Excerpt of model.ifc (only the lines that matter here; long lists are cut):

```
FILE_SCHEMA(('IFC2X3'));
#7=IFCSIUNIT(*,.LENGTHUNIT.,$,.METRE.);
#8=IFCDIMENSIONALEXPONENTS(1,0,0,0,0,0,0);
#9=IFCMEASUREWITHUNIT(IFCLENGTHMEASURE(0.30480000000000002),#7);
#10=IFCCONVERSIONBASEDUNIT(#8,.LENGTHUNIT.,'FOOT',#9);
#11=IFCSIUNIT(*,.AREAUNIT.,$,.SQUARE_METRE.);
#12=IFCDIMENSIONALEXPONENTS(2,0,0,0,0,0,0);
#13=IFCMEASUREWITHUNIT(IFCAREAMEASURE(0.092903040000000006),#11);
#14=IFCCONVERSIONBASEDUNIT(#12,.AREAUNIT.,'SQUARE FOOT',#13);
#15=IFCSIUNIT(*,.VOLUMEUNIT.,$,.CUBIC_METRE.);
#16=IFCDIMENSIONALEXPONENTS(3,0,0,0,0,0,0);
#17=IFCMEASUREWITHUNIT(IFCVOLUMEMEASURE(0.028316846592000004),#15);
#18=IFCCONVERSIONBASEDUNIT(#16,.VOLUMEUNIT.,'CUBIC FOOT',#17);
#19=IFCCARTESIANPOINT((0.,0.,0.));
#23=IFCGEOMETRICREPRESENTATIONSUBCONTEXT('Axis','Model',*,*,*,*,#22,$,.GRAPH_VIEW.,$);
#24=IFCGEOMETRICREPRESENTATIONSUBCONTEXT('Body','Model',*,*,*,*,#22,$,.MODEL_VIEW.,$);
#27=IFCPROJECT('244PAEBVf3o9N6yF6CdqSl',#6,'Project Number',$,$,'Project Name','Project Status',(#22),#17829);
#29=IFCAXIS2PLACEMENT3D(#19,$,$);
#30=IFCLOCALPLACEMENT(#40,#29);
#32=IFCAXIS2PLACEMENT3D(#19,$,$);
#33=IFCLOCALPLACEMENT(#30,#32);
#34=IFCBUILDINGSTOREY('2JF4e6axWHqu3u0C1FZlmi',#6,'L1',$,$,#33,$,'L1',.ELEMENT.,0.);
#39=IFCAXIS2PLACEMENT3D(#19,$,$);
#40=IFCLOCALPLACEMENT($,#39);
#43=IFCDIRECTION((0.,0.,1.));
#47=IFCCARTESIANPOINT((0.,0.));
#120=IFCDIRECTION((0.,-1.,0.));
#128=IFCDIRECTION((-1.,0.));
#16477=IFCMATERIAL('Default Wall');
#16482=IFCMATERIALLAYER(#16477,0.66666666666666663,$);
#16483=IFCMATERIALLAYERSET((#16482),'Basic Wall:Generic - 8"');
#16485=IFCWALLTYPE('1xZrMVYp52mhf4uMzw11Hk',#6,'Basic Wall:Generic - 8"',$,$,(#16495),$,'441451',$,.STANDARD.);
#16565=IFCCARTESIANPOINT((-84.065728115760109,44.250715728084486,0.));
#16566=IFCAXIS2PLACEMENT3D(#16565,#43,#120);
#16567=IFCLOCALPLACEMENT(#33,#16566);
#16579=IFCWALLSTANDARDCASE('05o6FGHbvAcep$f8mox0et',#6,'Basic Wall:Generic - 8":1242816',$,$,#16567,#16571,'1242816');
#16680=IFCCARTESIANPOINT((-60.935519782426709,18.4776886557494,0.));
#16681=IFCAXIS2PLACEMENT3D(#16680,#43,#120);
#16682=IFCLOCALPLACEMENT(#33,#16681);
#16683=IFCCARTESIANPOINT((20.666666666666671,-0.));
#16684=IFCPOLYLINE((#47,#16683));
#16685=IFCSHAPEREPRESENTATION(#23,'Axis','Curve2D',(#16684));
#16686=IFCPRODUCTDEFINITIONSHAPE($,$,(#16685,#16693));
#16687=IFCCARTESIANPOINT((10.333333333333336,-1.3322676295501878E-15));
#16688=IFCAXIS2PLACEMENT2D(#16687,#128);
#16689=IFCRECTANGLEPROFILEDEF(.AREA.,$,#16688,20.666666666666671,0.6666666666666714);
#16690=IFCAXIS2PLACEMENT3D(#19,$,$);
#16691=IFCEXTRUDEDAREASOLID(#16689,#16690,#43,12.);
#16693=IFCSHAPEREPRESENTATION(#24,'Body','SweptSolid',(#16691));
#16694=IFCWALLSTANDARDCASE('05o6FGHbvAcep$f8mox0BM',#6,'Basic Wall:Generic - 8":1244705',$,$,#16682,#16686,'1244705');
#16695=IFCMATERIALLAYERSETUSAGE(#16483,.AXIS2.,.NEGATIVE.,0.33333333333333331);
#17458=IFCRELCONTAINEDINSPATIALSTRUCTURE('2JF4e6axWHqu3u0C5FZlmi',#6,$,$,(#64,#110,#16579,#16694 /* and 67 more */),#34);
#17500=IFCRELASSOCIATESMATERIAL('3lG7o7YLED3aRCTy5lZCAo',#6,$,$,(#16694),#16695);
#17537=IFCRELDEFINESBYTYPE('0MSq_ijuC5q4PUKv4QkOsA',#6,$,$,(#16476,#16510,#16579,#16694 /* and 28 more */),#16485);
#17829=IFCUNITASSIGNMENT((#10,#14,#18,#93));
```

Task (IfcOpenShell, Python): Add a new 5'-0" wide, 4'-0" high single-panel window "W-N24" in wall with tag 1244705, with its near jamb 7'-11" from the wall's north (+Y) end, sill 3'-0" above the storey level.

```python
import numpy as np
import ifcopenshell
import ifcopenshell.api.feature
import ifcopenshell.api.geometry
import ifcopenshell.api.root
import ifcopenshell.api.spatial
import ifcopenshell.api.type
import ifcopenshell.geom
import ifcopenshell.util.element
import ifcopenshell.util.placement
import ifcopenshell.util.representation
import ifcopenshell.util.shape
import ifcopenshell.util.unit

model = ifcopenshell.open("model.ifc")
unit_scale = ifcopenshell.util.unit.calculate_unit_scale(model)
settings = ifcopenshell.geom.settings()


def volume(element):
    """Net volume in cubic metres, openings subtracted."""
    shape = ifcopenshell.geom.create_shape(settings, element)
    return ifcopenshell.util.shape.get_volume(shape.geometry)


wall = model.by_guid("05o6FGHbvAcep$f8mox0BM")
storey = ifcopenshell.util.element.get_container(wall, ifc_class="IfcBuildingStorey")
context = ifcopenshell.util.representation.get_context(model, "Model", "Body", "MODEL_VIEW")
before = volume(wall)

width, height, from_end, sill = 1.524, 1.2192, 2.413, 0.9144  # metres

# The wall runs along its own X axis, and the end named is its -X end.
wall_shape = ifcopenshell.geom.create_shape(settings, wall)
x, y, z = ifcopenshell.util.shape.get_vertices(wall_shape.geometry).T
start = x.min() + from_end
face, thickness = float(y.min()), float(y.max() - y.min())
wall_matrix = ifcopenshell.util.placement.get_local_placement(wall.ObjectPlacement)
level = ifcopenshell.util.placement.get_local_placement(storey.ObjectPlacement)[2, 3]


def in_wall(x, y):
    """Placement at x, y metres in the wall's axes, at sill height."""
    matrix = wall_matrix.copy()
    matrix[:, 3] = wall_matrix @ np.array([x / unit_scale, y / unit_scale, 0.0, 1.0])
    matrix[2, 3] = level + sill / unit_scale
    return matrix


# Opening: a box that overshoots both wall faces by 50 mm.
opening = ifcopenshell.api.root.create_entity(model, ifc_class="IfcOpeningElement")
box = ifcopenshell.api.geometry.add_wall_representation(
    model, context=context, length=width, height=height, thickness=thickness + 0.1
)
ifcopenshell.api.geometry.assign_representation(model, product=opening, representation=box)
ifcopenshell.api.geometry.edit_object_placement(model, product=opening, matrix=in_wall(start, face - 0.05), is_si=False)
ifcopenshell.api.feature.add_feature(model, feature=opening, element=wall)

window = ifcopenshell.api.root.create_entity(model, ifc_class="IfcWindow", name="W-N24")
window.OverallWidth, window.OverallHeight = width / unit_scale, height / unit_scale
body = ifcopenshell.api.geometry.add_window_representation(
    model,
    context=context,
    overall_width=window.OverallWidth,
    overall_height=window.OverallHeight,
    partition_type="SINGLE_PANEL",
)
ifcopenshell.api.geometry.assign_representation(model, product=window, representation=body)
ifcopenshell.api.spatial.assign_container(model, products=[window], relating_structure=storey)
fills = ifcopenshell.api.feature.add_filling(model, opening=opening, element=window)
fills.OwnerHistory = window.OwnerHistory  # required in IFC2X3

# IFC2X3 keeps the operation on the window style.
style = ifcopenshell.api.root.create_entity(model, ifc_class="IfcWindowStyle", name="W-N24")
style.OperationType, style.ConstructionType = "SINGLE_PANEL", "NOTDEFINED"
style.ParameterTakesPrecedence = style.Sizeable = False
ifcopenshell.api.type.assign_type(model, related_objects=[window], relating_type=style)

# Centre the window in the wall's thickness.
ifcopenshell.api.geometry.edit_object_placement(model, product=window, matrix=in_wall(start, face), is_si=False)
window_shape = ifcopenshell.geom.create_shape(settings, window)
depth = ifcopenshell.util.shape.get_vertices(window_shape.geometry)[:, 1]
offset = face + thickness / 2 - (depth.min() + depth.max()) / 2
ifcopenshell.api.geometry.edit_object_placement(model, product=window, matrix=in_wall(start, offset), is_si=False)

after = volume(wall)

print(f"wall volume {before:.3f} -> {after:.3f} m3")

model.write("model_v2.ifc")
```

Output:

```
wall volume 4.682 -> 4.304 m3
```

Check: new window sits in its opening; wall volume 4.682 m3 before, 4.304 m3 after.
